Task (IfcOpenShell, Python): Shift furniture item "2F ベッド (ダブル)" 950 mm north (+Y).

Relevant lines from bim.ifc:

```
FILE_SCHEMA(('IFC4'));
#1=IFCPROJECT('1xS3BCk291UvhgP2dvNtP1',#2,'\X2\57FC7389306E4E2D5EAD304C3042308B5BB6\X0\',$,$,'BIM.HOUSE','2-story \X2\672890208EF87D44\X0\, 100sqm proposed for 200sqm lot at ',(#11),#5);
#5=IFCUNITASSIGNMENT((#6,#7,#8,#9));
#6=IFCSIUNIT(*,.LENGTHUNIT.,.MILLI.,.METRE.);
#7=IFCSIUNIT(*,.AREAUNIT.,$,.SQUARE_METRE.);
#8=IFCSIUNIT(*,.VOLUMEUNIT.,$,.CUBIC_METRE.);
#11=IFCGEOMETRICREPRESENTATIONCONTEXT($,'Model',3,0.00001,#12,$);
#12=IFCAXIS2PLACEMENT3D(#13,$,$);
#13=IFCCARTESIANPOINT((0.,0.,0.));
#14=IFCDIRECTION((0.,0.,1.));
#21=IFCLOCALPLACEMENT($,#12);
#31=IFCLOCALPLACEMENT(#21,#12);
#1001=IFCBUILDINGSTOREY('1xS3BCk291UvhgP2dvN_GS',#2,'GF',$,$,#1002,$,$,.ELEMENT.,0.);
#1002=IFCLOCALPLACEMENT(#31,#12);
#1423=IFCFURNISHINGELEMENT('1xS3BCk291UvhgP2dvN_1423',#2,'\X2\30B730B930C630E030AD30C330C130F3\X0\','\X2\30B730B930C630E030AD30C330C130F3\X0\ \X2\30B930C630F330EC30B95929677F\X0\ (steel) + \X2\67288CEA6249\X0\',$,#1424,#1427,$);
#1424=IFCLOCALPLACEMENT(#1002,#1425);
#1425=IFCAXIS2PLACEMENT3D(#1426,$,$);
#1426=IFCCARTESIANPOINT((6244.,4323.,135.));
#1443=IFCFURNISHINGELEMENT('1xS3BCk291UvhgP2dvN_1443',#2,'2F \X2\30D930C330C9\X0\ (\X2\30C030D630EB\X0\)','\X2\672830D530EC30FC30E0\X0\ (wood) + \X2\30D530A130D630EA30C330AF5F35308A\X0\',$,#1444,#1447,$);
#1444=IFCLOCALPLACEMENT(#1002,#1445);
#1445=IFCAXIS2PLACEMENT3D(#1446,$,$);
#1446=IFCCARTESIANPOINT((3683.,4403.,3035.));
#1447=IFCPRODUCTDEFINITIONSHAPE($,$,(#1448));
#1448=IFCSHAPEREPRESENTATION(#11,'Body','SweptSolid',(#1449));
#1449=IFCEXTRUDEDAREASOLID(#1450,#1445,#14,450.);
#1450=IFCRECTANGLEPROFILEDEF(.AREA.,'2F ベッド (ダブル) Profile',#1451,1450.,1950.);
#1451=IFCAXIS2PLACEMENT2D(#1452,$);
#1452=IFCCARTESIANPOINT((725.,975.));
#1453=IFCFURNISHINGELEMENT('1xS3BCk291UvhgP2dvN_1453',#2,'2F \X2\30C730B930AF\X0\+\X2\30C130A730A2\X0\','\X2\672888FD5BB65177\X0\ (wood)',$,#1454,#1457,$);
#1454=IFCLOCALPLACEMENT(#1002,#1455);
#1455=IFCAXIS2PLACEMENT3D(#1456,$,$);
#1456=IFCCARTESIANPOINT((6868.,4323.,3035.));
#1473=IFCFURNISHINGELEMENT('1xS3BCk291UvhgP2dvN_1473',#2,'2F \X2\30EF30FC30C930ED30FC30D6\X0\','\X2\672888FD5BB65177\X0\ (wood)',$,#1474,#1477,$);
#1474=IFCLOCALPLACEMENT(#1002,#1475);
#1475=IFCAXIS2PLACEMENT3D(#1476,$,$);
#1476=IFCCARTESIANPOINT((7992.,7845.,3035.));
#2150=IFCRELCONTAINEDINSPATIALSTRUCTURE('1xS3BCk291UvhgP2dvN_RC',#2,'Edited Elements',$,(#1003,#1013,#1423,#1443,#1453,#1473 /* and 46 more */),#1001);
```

```python
import ifcopenshell
import ifcopenshell.api.geometry
import ifcopenshell.util.placement
import ifcopenshell.util.unit

model = ifcopenshell.open("bim.ifc")
unit_scale = ifcopenshell.util.unit.calculate_unit_scale(model)

item = model.by_guid("1xS3BCk291UvhgP2dvN_1443")
matrix = ifcopenshell.util.placement.get_local_placement(item.ObjectPlacement)
matrix[1, 3] += 0.95 / unit_scale
ifcopenshell.api.geometry.edit_object_placement(model, product=item, matrix=matrix, is_si=False)

print(ifcopenshell.util.placement.get_local_placement(item.ObjectPlacement).round(3) + 0.0)

model.write("bim_rev.ifc")
```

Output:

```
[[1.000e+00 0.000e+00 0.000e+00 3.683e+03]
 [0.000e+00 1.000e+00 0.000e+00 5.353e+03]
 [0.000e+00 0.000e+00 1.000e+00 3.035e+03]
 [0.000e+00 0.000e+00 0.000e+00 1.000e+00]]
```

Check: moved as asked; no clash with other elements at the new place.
